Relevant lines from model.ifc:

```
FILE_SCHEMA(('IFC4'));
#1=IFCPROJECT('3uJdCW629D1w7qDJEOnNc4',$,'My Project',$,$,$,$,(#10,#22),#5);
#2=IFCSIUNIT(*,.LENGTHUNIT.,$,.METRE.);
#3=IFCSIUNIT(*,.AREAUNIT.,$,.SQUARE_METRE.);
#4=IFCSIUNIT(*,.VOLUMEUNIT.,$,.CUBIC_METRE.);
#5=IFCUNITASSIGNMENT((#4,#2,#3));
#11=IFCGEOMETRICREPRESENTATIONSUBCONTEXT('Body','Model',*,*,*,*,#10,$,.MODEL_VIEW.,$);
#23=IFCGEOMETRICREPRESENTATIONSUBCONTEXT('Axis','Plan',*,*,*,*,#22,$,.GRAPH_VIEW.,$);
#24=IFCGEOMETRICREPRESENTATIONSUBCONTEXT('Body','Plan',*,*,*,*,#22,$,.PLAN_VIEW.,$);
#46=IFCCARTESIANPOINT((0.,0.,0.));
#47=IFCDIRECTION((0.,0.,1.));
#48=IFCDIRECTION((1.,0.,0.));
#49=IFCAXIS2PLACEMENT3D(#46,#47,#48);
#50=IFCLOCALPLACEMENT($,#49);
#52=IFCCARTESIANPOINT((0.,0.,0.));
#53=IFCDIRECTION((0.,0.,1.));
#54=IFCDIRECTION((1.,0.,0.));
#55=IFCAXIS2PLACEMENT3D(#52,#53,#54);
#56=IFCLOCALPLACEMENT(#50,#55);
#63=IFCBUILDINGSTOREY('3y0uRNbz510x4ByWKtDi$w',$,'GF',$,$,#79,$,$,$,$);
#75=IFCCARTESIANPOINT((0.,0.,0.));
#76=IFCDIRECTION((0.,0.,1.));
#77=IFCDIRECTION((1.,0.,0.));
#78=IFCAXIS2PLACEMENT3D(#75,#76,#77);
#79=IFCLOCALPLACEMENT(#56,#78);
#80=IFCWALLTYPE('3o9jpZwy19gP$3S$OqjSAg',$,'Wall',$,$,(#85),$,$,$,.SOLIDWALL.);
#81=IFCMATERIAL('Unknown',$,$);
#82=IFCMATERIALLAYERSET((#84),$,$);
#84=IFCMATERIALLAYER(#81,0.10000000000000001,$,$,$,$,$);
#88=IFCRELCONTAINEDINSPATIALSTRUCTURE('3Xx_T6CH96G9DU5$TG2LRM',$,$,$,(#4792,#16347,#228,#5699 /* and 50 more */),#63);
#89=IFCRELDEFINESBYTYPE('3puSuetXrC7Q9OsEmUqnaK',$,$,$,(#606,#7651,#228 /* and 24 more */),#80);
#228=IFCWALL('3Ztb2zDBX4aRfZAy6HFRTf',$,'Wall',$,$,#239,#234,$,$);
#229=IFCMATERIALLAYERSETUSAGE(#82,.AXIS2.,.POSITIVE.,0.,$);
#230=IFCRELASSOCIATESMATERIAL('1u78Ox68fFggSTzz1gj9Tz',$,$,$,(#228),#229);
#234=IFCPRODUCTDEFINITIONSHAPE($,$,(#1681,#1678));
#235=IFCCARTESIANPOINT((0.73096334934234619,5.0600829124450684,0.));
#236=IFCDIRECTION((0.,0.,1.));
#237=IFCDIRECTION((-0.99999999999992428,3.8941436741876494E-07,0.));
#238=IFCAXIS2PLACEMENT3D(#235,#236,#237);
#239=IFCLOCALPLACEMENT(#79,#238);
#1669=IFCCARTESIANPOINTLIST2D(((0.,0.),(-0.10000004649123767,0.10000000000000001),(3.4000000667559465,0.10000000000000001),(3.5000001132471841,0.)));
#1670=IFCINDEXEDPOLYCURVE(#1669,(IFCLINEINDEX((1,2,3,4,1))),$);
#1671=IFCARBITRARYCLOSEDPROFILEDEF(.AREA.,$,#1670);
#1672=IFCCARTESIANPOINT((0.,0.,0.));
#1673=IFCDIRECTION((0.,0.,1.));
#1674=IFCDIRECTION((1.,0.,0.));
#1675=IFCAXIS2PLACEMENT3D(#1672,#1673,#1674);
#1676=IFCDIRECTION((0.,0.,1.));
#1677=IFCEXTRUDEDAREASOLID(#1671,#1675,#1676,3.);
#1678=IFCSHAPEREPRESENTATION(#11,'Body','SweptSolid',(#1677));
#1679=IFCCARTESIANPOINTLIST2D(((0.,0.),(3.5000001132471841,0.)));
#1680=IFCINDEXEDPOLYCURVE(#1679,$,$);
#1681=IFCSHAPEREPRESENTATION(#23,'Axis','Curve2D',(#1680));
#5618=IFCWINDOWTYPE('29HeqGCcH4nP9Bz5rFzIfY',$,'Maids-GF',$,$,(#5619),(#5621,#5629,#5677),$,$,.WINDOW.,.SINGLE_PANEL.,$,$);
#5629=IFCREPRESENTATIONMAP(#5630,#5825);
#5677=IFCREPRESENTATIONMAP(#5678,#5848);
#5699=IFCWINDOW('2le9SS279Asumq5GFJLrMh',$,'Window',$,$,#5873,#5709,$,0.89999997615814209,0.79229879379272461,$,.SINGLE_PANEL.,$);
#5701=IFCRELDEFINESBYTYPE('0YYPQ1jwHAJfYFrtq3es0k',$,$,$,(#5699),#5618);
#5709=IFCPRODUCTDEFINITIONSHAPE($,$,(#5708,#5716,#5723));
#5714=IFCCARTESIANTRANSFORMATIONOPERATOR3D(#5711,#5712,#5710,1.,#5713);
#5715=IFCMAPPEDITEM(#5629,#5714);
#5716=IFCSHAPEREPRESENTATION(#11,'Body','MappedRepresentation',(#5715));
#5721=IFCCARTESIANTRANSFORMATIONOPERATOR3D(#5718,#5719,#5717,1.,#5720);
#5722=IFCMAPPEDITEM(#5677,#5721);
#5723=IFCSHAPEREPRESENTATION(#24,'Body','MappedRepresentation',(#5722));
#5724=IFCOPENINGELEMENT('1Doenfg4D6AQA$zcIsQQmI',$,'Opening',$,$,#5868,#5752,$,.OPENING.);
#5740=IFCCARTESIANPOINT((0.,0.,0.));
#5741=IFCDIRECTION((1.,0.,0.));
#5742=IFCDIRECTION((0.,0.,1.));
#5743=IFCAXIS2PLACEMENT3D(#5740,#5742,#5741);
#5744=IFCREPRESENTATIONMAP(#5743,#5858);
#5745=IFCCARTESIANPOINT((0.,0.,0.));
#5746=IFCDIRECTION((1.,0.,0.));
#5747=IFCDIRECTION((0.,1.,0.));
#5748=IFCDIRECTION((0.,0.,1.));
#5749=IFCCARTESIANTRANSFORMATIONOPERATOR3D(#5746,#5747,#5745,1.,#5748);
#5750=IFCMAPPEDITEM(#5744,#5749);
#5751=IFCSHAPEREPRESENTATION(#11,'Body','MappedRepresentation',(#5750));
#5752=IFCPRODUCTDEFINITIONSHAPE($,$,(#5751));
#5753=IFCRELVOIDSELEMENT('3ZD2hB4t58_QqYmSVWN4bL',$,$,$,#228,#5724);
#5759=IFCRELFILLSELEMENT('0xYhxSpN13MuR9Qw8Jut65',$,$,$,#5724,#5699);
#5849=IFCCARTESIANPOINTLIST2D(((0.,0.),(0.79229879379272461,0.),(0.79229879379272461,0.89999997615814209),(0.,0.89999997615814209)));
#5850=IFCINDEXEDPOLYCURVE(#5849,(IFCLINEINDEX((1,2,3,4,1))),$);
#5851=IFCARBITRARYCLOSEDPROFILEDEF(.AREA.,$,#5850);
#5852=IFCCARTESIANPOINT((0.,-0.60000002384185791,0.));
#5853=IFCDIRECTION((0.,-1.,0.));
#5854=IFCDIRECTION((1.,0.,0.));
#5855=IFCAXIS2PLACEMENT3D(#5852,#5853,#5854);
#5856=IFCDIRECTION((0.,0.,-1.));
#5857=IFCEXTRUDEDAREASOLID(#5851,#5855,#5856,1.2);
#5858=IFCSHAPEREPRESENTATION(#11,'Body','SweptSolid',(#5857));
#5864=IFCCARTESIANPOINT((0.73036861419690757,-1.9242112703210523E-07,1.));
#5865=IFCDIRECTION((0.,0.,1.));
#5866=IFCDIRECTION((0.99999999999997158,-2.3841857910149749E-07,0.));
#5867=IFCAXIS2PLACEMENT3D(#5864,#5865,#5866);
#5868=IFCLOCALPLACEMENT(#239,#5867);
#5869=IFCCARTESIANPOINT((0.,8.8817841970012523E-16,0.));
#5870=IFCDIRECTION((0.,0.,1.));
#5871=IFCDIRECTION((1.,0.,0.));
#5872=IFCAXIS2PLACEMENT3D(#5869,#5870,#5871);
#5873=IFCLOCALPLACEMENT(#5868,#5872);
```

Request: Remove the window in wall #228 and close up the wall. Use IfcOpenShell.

```python
import ifcopenshell
import ifcopenshell.api.feature
import ifcopenshell.api.root
import ifcopenshell.geom
import ifcopenshell.util.shape

model = ifcopenshell.open("model.ifc")
settings = ifcopenshell.geom.settings()


def volume(element):
    """Net volume in cubic metres, openings subtracted."""
    shape = ifcopenshell.geom.create_shape(settings, element)
    return ifcopenshell.util.shape.get_volume(shape.geometry)


window = model.by_guid("2le9SS279Asumq5GFJLrMh")
opening = window.FillsVoids[0].RelatingOpeningElement
wall = opening.VoidsElements[0].RelatingBuildingElement
before = volume(wall)

ifcopenshell.api.root.remove_product(model, product=window)
ifcopenshell.api.feature.remove_feature(model, feature=opening)

after = volume(wall)

print(f"wall volume {before:.3f} -> {after:.3f} m3")

model.write("model-out.ifc")
```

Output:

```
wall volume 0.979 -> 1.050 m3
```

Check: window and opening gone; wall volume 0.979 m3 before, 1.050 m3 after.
